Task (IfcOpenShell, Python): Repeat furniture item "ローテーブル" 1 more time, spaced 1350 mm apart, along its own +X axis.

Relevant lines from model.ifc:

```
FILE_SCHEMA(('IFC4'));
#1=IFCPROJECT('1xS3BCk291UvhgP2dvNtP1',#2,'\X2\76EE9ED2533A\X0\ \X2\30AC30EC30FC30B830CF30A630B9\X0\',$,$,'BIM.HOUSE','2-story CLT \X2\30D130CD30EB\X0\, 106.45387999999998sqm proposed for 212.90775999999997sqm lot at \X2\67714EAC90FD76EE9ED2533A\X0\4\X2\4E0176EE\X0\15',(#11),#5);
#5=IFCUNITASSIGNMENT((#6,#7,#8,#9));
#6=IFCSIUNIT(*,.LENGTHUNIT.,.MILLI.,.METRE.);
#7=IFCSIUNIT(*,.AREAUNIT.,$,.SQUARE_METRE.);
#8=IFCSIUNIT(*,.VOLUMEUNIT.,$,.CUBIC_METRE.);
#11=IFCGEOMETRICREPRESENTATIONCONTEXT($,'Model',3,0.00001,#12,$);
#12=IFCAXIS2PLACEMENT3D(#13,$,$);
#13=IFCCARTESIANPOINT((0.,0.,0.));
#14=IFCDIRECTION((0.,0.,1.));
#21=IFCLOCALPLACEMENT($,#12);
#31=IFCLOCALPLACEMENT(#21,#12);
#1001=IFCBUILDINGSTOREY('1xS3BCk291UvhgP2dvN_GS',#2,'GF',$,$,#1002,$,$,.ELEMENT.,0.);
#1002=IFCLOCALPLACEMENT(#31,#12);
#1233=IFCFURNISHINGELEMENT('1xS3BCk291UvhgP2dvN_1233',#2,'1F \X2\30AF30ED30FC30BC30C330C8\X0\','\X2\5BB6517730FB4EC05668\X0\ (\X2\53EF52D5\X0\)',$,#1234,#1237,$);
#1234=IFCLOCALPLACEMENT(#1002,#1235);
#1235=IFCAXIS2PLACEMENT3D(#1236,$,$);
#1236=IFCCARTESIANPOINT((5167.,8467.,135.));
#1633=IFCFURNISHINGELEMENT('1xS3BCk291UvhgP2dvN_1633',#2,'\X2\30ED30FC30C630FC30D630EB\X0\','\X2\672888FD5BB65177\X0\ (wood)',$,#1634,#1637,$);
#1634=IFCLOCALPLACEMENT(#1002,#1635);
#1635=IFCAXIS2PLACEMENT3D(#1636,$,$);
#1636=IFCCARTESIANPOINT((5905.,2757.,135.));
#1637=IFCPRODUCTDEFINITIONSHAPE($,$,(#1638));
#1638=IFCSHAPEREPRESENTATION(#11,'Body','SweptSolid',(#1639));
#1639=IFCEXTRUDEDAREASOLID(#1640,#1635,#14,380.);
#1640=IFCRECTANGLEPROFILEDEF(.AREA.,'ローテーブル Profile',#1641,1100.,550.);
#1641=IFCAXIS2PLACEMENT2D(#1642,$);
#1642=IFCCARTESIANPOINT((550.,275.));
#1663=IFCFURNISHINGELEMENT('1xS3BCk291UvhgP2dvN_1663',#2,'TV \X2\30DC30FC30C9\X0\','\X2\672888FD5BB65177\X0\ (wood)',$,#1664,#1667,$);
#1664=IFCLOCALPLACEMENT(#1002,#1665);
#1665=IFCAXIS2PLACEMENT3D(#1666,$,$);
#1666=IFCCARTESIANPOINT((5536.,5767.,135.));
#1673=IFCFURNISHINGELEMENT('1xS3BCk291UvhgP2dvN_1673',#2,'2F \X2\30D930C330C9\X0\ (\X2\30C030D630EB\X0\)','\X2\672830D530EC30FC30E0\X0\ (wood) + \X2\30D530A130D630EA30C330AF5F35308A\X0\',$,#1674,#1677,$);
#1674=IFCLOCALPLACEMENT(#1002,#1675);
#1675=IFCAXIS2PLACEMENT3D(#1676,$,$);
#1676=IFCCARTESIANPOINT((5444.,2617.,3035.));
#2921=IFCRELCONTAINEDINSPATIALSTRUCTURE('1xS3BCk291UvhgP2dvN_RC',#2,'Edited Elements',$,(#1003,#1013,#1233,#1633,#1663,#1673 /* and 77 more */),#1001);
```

```python
import ifcopenshell
import ifcopenshell.api.geometry
import ifcopenshell.api.root
import ifcopenshell.util.element
import ifcopenshell.util.placement
import ifcopenshell.util.unit

model = ifcopenshell.open("model.ifc")
unit_scale = ifcopenshell.util.unit.calculate_unit_scale(model)


def reuse_history(source, copy):
    """copy_class also copies each property set's owner history, people and application; keep the originals."""
    for rel in copy.IsDefinedBy:
        if rel.is_a("IfcRelDefinesByProperties") and (history := rel.RelatingPropertyDefinition.OwnerHistory):
            rel.RelatingPropertyDefinition.OwnerHistory = source.OwnerHistory
            ifcopenshell.util.element.remove_deep2(model, history)


source = model.by_guid("1xS3BCk291UvhgP2dvN_1633")
base = ifcopenshell.util.placement.get_local_placement(source.ObjectPlacement)
step = base[:3, 0] * 1.35 / unit_scale

for i in range(1, 2):
    copy = ifcopenshell.api.root.copy_class(model, product=source)
    copy.Representation = ifcopenshell.util.element.copy_deep(
        model, source.Representation, exclude=["IfcGeometricRepresentationContext", "IfcRepresentationMap"]
    )
    reuse_history(source, copy)
    matrix = base.copy()
    matrix[:3, 3] += i * step
    print("added at", matrix[:3, 3].round(3) + 0.0)
    ifcopenshell.api.geometry.edit_object_placement(model, product=copy, matrix=matrix, is_si=False)

model.write("model-out.ifc")
```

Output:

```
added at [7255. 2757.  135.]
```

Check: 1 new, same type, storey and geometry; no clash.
